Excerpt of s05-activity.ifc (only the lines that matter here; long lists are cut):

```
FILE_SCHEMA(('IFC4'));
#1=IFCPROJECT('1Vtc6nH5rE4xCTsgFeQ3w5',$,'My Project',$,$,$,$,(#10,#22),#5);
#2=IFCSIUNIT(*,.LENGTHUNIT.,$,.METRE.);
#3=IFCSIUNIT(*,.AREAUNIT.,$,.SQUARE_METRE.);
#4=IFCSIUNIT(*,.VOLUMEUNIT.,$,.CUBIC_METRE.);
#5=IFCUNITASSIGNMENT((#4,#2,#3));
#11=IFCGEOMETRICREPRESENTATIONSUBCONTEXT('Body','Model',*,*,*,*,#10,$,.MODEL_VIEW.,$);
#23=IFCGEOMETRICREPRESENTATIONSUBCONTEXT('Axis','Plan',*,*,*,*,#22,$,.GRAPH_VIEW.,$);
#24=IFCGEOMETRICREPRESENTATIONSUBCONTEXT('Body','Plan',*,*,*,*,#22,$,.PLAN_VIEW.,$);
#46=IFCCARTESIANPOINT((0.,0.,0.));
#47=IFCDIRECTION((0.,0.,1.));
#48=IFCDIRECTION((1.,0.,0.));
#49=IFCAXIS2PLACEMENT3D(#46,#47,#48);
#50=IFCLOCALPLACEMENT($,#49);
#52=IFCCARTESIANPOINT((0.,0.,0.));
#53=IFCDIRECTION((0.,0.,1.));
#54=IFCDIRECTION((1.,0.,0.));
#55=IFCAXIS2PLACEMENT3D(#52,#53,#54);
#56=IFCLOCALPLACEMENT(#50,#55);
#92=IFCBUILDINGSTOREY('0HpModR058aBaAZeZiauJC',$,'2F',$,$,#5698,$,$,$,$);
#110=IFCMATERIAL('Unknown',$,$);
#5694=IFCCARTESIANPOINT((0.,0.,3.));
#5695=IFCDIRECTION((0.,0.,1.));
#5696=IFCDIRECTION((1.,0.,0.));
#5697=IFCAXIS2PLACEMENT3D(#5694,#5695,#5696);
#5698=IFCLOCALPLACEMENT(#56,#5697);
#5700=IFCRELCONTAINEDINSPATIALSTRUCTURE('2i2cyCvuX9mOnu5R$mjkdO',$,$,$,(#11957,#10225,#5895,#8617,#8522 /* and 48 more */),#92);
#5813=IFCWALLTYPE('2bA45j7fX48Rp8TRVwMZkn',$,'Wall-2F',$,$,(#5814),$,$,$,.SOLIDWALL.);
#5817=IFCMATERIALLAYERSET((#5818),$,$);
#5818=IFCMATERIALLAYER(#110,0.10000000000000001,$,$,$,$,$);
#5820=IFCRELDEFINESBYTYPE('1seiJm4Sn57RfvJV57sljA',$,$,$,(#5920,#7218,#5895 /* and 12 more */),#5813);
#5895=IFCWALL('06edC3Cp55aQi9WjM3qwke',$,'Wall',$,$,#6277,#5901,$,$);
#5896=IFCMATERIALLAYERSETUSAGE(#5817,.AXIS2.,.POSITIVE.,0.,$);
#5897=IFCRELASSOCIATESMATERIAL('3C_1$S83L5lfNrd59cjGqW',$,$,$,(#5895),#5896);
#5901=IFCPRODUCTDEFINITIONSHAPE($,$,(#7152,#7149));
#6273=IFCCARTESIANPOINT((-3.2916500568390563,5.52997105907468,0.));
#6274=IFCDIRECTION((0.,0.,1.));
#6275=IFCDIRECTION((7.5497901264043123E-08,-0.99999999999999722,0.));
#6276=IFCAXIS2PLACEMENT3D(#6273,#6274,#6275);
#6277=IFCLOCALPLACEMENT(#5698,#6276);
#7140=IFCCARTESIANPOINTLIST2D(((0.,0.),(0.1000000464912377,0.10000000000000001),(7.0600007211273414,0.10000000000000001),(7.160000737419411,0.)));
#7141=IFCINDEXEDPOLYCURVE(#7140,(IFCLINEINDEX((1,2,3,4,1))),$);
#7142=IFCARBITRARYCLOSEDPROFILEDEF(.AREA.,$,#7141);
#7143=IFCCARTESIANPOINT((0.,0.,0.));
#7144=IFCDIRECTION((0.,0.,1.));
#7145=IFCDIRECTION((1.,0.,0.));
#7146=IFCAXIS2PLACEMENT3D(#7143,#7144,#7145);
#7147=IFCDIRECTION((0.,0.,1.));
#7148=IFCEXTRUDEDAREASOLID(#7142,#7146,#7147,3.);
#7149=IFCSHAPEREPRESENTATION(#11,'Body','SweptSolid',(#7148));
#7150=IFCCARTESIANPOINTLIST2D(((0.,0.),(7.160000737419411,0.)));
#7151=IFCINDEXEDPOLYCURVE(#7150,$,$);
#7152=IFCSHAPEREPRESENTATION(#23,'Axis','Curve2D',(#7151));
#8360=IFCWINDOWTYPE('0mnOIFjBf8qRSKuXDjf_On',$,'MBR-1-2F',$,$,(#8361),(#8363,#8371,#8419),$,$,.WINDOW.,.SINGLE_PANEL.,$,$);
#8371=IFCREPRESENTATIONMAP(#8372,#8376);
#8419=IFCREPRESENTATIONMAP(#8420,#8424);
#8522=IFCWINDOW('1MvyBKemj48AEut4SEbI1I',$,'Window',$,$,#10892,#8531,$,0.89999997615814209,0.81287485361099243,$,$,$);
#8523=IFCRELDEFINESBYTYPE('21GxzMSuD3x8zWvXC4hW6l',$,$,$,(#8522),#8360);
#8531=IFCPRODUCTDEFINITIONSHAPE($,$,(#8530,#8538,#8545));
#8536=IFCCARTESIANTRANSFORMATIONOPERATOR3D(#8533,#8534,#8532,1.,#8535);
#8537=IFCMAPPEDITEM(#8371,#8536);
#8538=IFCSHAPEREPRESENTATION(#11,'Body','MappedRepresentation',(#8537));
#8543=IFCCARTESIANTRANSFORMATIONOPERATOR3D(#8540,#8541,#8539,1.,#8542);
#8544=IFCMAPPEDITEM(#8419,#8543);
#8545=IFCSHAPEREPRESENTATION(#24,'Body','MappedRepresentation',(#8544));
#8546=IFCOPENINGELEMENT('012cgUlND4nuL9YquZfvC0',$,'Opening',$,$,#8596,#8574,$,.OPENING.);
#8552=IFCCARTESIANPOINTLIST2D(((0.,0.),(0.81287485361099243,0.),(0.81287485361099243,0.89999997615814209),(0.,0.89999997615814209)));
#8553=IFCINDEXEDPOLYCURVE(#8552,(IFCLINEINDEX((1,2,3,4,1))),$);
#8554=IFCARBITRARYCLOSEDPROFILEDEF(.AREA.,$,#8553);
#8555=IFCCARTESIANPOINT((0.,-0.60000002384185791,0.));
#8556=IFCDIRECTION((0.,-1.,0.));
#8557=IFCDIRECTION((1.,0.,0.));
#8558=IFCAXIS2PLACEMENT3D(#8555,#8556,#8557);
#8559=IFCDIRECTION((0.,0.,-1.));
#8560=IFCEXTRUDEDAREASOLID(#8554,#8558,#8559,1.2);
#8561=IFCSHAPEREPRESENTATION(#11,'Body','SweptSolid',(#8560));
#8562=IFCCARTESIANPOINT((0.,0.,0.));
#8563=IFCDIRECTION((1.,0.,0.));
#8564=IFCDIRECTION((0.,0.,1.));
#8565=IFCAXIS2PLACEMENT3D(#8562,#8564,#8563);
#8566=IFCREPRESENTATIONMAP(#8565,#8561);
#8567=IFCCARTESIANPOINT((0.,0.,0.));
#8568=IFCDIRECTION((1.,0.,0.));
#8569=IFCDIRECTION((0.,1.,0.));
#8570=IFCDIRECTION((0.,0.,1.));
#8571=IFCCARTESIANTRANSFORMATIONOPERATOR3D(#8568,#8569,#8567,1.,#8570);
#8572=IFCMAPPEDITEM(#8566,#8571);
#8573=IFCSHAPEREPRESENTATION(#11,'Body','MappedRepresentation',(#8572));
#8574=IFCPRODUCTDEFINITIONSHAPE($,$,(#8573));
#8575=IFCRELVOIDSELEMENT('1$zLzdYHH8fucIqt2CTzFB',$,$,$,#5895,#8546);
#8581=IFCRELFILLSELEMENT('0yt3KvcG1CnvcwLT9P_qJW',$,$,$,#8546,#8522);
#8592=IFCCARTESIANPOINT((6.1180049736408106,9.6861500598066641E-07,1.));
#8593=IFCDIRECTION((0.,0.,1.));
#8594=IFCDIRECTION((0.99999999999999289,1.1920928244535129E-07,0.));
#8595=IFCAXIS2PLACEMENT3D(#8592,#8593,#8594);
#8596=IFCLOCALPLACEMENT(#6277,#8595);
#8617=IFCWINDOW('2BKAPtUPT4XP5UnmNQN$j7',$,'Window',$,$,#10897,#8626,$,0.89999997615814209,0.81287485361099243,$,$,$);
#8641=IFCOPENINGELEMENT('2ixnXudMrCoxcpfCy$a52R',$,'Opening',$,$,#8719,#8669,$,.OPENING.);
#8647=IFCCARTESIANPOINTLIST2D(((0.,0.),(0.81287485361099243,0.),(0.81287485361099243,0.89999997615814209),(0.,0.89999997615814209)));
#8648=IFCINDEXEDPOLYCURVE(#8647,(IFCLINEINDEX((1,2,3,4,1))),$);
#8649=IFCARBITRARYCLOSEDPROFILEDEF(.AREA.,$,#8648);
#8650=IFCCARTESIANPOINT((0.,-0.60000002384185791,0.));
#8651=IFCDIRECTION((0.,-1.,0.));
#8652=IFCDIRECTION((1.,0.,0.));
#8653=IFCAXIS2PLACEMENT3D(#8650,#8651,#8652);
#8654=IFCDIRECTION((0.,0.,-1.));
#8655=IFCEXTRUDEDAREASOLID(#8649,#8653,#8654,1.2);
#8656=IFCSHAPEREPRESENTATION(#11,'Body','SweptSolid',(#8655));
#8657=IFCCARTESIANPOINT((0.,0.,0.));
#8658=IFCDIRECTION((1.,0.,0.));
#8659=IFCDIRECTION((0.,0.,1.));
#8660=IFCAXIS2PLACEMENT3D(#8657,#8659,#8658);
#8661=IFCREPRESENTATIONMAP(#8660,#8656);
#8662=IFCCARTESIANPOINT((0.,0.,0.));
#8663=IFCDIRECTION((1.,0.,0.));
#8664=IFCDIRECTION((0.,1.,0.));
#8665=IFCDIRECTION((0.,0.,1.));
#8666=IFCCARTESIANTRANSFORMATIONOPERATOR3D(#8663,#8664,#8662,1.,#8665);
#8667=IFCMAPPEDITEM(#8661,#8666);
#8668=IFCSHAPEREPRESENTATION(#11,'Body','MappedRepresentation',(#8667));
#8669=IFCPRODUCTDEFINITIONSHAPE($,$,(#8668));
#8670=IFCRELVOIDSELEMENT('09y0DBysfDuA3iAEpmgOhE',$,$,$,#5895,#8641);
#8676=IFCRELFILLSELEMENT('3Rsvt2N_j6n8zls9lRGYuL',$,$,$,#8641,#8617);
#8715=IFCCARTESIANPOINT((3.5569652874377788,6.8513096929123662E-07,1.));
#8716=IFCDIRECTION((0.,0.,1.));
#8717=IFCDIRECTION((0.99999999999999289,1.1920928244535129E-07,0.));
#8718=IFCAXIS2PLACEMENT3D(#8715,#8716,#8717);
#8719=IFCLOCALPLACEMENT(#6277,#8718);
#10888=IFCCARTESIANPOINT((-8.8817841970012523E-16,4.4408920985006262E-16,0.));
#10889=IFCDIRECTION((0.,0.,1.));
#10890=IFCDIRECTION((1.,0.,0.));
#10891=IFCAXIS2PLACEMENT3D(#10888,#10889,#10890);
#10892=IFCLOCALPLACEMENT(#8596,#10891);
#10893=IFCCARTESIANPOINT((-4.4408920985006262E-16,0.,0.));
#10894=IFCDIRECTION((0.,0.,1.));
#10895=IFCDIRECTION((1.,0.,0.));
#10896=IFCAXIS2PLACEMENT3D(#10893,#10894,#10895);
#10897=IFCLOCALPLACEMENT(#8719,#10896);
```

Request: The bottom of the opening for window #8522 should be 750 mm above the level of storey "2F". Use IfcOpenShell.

```python
import numpy as np
import ifcopenshell
import ifcopenshell.api.geometry
import ifcopenshell.geom
import ifcopenshell.util.element
import ifcopenshell.util.placement
import ifcopenshell.util.shape
import ifcopenshell.util.unit

model = ifcopenshell.open("s05-activity.ifc")
unit_scale = ifcopenshell.util.unit.calculate_unit_scale(model)

window = model.by_guid("1MvyBKemj48AEut4SEbI1I")
opening = window.FillsVoids[0].RelatingOpeningElement
storey = ifcopenshell.util.element.get_container(window, ifc_class="IfcBuildingStorey")
level = ifcopenshell.util.placement.get_local_placement(storey.ObjectPlacement)[2, 3]

# The opening's origin need not be at the sill, so measure its lowest point.
shape = ifcopenshell.geom.create_shape(ifcopenshell.geom.settings(), opening)
bottom = ifcopenshell.util.shape.get_shape_bottom_elevation(shape, shape.geometry) / unit_scale
dz = level + 0.75 - bottom

shift = np.array([0.0, 0.0, dz])
# The window is placed relative to its opening, so it follows when the opening moves.
matrix = ifcopenshell.util.placement.get_local_placement(opening.ObjectPlacement)
matrix[:3, 3] += shift
ifcopenshell.api.geometry.edit_object_placement(
    model, product=opening, matrix=matrix, is_si=False, should_transform_children=True
)

print(f"moved by {dz * unit_scale:+.3f} m")

model.write("s05-activity_edited.ifc")
```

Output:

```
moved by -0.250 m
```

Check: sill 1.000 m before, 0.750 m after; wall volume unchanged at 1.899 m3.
